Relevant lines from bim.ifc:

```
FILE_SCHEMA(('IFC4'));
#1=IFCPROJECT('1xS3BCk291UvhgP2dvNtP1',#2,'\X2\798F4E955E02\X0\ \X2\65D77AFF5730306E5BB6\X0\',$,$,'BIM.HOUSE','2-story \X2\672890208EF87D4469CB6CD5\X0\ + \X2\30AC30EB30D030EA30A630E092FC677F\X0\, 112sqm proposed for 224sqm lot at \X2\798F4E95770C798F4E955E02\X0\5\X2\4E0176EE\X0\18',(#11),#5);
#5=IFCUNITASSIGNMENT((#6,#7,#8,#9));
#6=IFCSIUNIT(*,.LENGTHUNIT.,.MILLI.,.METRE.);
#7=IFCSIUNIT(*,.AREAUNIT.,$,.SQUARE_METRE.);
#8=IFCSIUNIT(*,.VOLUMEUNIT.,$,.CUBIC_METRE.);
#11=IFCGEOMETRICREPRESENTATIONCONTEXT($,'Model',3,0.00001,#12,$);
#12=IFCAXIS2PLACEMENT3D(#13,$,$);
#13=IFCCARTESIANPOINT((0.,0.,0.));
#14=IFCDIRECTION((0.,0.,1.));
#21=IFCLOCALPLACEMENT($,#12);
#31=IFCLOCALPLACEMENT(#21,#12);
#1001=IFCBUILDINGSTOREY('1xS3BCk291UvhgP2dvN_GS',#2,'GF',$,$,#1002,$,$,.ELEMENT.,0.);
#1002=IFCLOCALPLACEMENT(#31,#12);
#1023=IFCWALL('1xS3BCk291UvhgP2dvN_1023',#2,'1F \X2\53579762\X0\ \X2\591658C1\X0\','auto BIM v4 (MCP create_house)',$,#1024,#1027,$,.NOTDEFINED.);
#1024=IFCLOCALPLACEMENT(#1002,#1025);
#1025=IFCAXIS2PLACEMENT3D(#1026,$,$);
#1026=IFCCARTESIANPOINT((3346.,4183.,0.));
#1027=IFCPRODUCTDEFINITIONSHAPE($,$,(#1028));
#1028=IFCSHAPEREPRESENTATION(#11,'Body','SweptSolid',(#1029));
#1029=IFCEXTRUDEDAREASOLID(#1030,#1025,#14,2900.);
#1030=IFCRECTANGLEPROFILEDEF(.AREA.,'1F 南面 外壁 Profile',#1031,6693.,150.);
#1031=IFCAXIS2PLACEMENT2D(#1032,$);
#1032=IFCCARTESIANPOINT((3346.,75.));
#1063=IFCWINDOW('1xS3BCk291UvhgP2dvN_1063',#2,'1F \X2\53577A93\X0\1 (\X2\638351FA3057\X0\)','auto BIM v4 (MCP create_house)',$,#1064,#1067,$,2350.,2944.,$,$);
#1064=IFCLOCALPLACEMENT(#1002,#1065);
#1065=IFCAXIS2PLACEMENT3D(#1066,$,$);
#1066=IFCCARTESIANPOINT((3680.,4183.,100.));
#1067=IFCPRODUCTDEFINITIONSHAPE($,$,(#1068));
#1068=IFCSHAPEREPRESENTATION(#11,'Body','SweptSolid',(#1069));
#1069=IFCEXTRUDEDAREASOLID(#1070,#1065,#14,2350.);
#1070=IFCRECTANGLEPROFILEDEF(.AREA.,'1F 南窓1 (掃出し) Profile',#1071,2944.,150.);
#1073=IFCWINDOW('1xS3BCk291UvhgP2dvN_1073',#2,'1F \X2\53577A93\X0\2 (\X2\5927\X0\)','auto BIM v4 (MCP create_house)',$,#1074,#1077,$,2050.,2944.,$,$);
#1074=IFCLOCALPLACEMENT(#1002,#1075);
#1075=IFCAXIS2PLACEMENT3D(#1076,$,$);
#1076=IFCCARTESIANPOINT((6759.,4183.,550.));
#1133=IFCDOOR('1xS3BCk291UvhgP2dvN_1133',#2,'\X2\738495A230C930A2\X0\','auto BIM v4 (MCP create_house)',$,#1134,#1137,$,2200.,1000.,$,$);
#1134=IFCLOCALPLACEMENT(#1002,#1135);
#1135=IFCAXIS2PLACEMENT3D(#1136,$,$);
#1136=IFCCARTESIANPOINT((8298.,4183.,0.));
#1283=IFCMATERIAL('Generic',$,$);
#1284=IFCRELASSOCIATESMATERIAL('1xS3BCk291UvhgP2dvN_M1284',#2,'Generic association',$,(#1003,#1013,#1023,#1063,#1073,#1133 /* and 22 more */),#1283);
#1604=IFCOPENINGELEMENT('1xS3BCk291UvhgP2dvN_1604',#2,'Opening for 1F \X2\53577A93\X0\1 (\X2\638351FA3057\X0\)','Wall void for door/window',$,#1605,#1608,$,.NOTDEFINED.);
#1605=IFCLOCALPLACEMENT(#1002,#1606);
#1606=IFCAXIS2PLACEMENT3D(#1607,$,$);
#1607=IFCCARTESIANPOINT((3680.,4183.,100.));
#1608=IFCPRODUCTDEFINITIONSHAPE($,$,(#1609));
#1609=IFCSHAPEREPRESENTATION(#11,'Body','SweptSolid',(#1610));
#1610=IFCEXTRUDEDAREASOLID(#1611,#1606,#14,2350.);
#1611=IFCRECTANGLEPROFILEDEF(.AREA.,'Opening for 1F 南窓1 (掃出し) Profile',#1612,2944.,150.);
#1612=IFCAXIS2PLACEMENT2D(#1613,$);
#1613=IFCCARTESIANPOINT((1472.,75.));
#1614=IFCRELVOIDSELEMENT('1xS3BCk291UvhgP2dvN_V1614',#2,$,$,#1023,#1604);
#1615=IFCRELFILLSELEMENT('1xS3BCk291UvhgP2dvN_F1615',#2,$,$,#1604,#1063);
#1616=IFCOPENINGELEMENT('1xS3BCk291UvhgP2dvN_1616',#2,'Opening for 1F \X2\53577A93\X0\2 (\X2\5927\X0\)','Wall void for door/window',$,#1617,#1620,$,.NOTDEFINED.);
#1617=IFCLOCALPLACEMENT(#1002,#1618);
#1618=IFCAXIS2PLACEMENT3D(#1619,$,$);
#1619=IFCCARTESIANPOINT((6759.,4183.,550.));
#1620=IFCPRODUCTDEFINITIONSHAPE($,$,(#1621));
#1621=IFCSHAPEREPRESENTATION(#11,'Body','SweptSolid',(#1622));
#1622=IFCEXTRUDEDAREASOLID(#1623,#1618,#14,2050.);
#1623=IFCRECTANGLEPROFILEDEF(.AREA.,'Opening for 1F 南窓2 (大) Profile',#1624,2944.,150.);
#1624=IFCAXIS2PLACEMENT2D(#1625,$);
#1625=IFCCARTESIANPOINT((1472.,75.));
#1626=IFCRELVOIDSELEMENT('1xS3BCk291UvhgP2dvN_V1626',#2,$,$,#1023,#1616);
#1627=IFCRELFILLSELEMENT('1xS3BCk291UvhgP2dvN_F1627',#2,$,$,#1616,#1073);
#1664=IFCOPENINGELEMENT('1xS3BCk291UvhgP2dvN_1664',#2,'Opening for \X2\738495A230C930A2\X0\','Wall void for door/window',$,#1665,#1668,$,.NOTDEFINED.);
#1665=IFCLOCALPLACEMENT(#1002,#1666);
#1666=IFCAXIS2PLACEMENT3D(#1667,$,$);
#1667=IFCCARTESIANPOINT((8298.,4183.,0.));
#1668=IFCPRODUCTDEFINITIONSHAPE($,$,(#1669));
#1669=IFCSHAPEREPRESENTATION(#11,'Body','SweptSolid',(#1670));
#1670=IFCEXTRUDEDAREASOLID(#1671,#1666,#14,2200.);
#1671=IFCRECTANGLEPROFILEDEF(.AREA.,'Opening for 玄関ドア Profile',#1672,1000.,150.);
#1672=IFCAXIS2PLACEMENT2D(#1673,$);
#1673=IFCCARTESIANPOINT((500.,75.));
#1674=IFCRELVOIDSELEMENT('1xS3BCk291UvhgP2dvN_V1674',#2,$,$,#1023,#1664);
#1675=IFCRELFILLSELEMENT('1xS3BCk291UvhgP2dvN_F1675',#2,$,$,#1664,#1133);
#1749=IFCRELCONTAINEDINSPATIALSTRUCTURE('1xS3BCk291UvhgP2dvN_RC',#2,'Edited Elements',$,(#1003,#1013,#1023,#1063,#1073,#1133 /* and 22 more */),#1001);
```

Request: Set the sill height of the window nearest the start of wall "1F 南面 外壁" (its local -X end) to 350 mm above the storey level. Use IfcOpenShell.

```python
import numpy as np
import ifcopenshell
import ifcopenshell.api.geometry
import ifcopenshell.geom
import ifcopenshell.util.element
import ifcopenshell.util.placement
import ifcopenshell.util.shape
import ifcopenshell.util.unit

model = ifcopenshell.open("bim.ifc")
unit_scale = ifcopenshell.util.unit.calculate_unit_scale(model)

window = model.by_guid("1xS3BCk291UvhgP2dvN_1063")
opening = window.FillsVoids[0].RelatingOpeningElement
storey = ifcopenshell.util.element.get_container(window, ifc_class="IfcBuildingStorey")
level = ifcopenshell.util.placement.get_local_placement(storey.ObjectPlacement)[2, 3]

# The opening's origin need not be at the sill, so measure its lowest point.
shape = ifcopenshell.geom.create_shape(ifcopenshell.geom.settings(), opening)
bottom = ifcopenshell.util.shape.get_shape_bottom_elevation(shape, shape.geometry) / unit_scale
dz = level + 350.0 - bottom

shift = np.array([0.0, 0.0, dz])
# The window is not placed relative to its opening, so move both.
for product in (opening, window):
    matrix = ifcopenshell.util.placement.get_local_placement(product.ObjectPlacement)
    matrix[:3, 3] += shift
    ifcopenshell.api.geometry.edit_object_placement(model, product=product, matrix=matrix, is_si=False)

print(f"moved by {dz * unit_scale:+.3f} m")

model.write("bim_updated.ifc")
```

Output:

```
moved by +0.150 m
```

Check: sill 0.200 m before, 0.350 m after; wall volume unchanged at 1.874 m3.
